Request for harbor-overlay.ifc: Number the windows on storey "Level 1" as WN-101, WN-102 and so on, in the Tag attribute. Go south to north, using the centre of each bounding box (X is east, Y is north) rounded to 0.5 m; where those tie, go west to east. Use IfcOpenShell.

First a look at what the model holds.

```python
import ifcopenshell
import ifcopenshell.util.element
import ifcopenshell.util.placement

model = ifcopenshell.open("harbor-overlay.ifc")
print(model.schema)
storey = next(s for s in model.by_type("IfcBuildingStorey") if s.Name == "Level 1")
windows = [e for e in ifcopenshell.util.element.get_decomposition(storey) if e.is_a("IfcWindow")]
for e in sorted(windows, key=lambda e: e.id()):
    origin = ifcopenshell.util.placement.get_local_placement(e.ObjectPlacement)[:3, 3]
    print(e.id(), e.Tag, e.Name, origin.round(2) + 0.0, sep=" | ")
```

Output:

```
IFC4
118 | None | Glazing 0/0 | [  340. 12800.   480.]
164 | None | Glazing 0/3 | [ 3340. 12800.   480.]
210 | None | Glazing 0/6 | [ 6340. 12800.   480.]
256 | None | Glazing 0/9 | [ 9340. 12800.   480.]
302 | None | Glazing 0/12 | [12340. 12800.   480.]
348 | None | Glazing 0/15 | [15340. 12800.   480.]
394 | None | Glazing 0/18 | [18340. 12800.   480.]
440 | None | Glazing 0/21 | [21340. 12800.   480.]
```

```python
import ifcopenshell
import ifcopenshell.geom
import ifcopenshell.util.element
import ifcopenshell.util.shape

model = ifcopenshell.open("harbor-overlay.ifc")
settings = ifcopenshell.geom.settings()
settings.set("use-world-coords", True)


def centre(element):
    shape = ifcopenshell.geom.create_shape(settings, element)
    return ifcopenshell.util.shape.get_bbox_centroid(shape.geometry)


storey = next(s for s in model.by_type("IfcBuildingStorey") if s.Name == "Level 1")
windows = [e for e in ifcopenshell.util.element.get_decomposition(storey) if e.is_a("IfcWindow")]

# Insertion points can sit at a corner or the storey origin, so sort by the geometry (in metres).
centres = {e: centre(e) for e in windows}
windows.sort(key=lambda e: (round(centres[e][1] / 0.5), centres[e][0]))

for i, e in enumerate(windows, start=1):
    number = f"WN-1{i:02d}"
    e.Tag = number
    print(e.id(), number)

model.write("harbor-overlay_updated.ifc")
```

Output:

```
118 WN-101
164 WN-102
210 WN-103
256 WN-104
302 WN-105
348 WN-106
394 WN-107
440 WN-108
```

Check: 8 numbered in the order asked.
